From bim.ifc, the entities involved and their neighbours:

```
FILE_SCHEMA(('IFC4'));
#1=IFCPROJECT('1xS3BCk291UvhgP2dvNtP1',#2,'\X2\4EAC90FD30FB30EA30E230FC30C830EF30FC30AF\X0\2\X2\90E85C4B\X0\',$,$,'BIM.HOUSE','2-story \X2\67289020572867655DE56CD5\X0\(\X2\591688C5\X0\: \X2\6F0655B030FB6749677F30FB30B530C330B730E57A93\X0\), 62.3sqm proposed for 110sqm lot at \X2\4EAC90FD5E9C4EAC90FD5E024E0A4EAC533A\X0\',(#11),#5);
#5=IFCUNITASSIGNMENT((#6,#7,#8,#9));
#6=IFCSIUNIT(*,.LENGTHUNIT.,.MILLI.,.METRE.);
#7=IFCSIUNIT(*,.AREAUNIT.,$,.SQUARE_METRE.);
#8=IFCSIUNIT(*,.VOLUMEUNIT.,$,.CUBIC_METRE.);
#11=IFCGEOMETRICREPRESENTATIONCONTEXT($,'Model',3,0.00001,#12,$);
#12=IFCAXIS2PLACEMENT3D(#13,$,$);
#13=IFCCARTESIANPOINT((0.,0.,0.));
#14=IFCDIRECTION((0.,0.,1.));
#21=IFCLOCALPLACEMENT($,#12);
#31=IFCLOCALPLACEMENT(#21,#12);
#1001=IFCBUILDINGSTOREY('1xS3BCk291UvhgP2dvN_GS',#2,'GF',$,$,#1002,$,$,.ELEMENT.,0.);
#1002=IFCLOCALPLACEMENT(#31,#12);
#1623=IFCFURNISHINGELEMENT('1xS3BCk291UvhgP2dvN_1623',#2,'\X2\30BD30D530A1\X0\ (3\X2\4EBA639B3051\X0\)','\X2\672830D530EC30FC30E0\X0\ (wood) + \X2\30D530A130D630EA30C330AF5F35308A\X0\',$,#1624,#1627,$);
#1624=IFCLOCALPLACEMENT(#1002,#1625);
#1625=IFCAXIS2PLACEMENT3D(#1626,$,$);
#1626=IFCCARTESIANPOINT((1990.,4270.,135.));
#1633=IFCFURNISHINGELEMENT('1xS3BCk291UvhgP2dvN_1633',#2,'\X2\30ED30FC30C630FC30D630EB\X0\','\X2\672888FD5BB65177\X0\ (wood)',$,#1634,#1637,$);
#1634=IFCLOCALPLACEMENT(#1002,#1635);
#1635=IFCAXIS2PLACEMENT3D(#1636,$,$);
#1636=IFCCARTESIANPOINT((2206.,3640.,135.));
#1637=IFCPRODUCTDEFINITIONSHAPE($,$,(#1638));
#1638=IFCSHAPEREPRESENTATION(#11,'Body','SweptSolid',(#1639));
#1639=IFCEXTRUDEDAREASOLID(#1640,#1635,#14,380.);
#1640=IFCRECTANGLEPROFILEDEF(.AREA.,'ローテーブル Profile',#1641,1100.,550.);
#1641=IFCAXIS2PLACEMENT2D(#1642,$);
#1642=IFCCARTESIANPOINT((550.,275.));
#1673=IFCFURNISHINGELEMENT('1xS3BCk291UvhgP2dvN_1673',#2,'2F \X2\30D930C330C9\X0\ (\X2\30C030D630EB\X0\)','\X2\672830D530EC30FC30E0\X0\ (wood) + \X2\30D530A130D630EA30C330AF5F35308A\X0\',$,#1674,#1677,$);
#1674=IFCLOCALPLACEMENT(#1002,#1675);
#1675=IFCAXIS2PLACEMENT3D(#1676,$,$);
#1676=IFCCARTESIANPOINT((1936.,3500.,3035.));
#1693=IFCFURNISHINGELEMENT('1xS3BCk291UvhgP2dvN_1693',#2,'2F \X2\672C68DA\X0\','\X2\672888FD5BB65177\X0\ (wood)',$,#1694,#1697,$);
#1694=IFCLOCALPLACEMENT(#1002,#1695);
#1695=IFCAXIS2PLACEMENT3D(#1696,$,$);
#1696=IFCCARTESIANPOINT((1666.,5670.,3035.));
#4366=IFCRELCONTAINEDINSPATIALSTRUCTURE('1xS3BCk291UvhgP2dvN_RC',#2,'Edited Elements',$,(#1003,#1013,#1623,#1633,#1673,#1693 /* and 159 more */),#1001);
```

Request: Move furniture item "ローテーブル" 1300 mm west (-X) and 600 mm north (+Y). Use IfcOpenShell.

```python
import ifcopenshell
import ifcopenshell.api.geometry
import ifcopenshell.util.placement

model = ifcopenshell.open("bim.ifc")

item = model.by_guid("1xS3BCk291UvhgP2dvN_1633")
matrix = ifcopenshell.util.placement.get_local_placement(item.ObjectPlacement)
matrix[0, 3] -= 1300.0
matrix[1, 3] += 600.0
ifcopenshell.api.geometry.edit_object_placement(model, product=item, matrix=matrix, is_si=False)

print(ifcopenshell.util.placement.get_local_placement(item.ObjectPlacement).round(3) + 0.0)

model.write("bim_v2.ifc")
```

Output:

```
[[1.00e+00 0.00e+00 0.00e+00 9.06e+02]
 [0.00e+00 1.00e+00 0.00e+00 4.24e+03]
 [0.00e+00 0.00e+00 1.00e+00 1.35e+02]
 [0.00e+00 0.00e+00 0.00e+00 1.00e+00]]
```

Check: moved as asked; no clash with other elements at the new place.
